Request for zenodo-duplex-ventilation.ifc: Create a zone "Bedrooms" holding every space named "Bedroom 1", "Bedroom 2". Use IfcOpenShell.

First a look at what the model holds.

```python
import ifcopenshell

model = ifcopenshell.open("zenodo-duplex-ventilation.ifc")
print(model.schema)
seen = {}
for space in model.by_type("IfcSpace"):
    seen[space.LongName] = seen.get(space.LongName, 0) + 1
for name, count in sorted(seen.items(), key=str):
    print(count, "x", name)
print("zones:", [z.Name for z in model.by_type("IfcZone")][:20])
```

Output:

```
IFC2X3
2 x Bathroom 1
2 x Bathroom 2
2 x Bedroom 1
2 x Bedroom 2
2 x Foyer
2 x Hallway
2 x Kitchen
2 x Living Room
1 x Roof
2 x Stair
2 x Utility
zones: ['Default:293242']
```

```python
import ifcopenshell
import ifcopenshell.api.group
import ifcopenshell.api.root

model = ifcopenshell.open("zenodo-duplex-ventilation.ifc")

names = {"Bedroom 1", "Bedroom 2"}
spaces = [s for s in model.by_type("IfcSpace") if s.LongName in names]

zone = ifcopenshell.api.root.create_entity(model, ifc_class="IfcZone", name="Bedrooms")
ifcopenshell.api.group.assign_group(model, products=spaces, group=zone)
print(len(spaces), "spaces in", zone.Name)

model.write("zenodo-duplex-ventilation_rev.ifc")
```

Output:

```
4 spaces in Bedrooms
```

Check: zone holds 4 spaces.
